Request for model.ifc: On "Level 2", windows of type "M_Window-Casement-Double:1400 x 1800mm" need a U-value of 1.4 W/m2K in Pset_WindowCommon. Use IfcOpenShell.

First a look at what the model holds.

```python
import ifcopenshell
import ifcopenshell.util.element

model = ifcopenshell.open("model.ifc")
print(model.schema)
storey = next(s for s in model.by_type("IfcBuildingStorey") if s.Name == "Level 2")
windows = [e for e in ifcopenshell.util.element.get_decomposition(storey) if e.is_a("IfcWindow")]
seen = {}
for e in windows:
    element_type = ifcopenshell.util.element.get_type(e)
    key = (element_type.Name if element_type != e and element_type else None, ifcopenshell.util.element.get_pset(e, "Pset_WindowCommon", "ThermalTransmittance"))
    seen[key] = seen.get(key, 0) + 1
for (name, value), count in sorted(seen.items(), key=str):
    print(count, "x", name, "|", value)
```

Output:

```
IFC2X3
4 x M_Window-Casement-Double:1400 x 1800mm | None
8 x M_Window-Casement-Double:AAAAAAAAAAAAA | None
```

```python
import ifcopenshell
import ifcopenshell.api.pset
import ifcopenshell.util.element

model = ifcopenshell.open("model.ifc")

storey = next(s for s in model.by_type("IfcBuildingStorey") if s.Name == "Level 2")
windows = [e for e in ifcopenshell.util.element.get_decomposition(storey) if e.is_a("IfcWindow")]

count = 0
for e in windows:
    element_type = ifcopenshell.util.element.get_type(e)
    if element_type in (None, e) or element_type.Name != "M_Window-Casement-Double:1400 x 1800mm":
        continue
    # add_pset returns the element's existing set when there is one.
    pset = ifcopenshell.api.pset.add_pset(model, product=e, name="Pset_WindowCommon")
    ifcopenshell.api.pset.edit_pset(model, pset=pset, properties={"ThermalTransmittance": 1.4})
    count += 1

print(count, "windows updated")

model.write("model_updated.ifc")
```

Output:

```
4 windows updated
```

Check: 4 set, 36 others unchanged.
